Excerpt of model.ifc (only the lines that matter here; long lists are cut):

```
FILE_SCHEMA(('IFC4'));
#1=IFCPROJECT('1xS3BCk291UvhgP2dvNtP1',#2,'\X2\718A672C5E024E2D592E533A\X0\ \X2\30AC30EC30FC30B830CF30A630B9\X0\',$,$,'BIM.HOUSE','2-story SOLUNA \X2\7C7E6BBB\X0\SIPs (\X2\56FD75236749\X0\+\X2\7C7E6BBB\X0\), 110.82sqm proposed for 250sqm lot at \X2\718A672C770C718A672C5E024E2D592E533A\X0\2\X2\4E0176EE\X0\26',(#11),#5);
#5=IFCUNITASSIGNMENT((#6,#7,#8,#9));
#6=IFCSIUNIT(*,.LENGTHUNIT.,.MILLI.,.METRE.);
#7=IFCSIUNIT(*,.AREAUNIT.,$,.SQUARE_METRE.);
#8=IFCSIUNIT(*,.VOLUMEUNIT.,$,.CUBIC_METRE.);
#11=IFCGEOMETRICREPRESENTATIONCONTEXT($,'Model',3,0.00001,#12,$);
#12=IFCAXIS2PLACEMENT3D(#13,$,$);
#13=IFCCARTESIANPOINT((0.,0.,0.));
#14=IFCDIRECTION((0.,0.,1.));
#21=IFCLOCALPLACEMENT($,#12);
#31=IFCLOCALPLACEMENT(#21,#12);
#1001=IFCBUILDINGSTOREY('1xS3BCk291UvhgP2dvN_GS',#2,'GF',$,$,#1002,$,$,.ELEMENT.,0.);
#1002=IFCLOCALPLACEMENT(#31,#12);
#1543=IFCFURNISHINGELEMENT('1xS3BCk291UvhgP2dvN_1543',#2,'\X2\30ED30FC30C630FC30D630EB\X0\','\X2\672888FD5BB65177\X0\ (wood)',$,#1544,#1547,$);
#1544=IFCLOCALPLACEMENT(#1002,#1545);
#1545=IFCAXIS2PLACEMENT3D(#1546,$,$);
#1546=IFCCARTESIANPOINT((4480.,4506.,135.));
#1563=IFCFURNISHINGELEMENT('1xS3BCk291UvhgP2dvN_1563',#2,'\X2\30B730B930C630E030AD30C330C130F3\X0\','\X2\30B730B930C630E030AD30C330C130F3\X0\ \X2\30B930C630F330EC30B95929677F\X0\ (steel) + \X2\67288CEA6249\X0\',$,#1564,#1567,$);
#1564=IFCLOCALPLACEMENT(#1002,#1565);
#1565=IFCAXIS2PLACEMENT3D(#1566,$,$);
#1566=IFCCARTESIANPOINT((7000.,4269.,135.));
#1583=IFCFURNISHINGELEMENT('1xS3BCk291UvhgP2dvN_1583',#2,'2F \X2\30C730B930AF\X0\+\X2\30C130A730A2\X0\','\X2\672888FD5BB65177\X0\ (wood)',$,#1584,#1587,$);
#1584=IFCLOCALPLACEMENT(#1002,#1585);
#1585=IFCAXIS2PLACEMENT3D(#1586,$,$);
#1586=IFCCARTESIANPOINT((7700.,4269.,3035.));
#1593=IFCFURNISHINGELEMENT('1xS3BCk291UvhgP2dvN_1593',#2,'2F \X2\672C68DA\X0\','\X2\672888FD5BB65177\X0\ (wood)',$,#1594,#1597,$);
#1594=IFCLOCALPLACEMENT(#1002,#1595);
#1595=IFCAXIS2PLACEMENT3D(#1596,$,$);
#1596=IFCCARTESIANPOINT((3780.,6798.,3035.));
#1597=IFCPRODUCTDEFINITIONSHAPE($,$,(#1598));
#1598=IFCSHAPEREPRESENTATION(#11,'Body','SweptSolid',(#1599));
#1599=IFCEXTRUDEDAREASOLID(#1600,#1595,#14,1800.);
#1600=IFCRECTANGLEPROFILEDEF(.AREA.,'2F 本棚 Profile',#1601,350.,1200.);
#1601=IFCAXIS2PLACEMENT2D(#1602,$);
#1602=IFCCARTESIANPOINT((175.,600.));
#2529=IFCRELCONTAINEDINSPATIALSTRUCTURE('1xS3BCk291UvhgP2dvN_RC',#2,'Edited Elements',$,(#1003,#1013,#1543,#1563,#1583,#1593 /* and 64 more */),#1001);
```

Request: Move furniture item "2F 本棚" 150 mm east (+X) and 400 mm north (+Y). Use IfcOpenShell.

```python
import ifcopenshell
import ifcopenshell.api.geometry
import ifcopenshell.util.placement

model = ifcopenshell.open("model.ifc")

item = model.by_id(1593)
matrix = ifcopenshell.util.placement.get_local_placement(item.ObjectPlacement)
matrix[0, 3] += 150.0
matrix[1, 3] += 400.0
ifcopenshell.api.geometry.edit_object_placement(model, product=item, matrix=matrix, is_si=False)

print(ifcopenshell.util.placement.get_local_placement(item.ObjectPlacement).round(3) + 0.0)

model.write("model_updated.ifc")
```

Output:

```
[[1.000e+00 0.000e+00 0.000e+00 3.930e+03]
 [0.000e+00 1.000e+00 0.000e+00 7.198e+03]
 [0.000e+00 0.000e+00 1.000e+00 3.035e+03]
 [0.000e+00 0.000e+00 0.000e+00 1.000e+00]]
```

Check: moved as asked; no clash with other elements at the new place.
